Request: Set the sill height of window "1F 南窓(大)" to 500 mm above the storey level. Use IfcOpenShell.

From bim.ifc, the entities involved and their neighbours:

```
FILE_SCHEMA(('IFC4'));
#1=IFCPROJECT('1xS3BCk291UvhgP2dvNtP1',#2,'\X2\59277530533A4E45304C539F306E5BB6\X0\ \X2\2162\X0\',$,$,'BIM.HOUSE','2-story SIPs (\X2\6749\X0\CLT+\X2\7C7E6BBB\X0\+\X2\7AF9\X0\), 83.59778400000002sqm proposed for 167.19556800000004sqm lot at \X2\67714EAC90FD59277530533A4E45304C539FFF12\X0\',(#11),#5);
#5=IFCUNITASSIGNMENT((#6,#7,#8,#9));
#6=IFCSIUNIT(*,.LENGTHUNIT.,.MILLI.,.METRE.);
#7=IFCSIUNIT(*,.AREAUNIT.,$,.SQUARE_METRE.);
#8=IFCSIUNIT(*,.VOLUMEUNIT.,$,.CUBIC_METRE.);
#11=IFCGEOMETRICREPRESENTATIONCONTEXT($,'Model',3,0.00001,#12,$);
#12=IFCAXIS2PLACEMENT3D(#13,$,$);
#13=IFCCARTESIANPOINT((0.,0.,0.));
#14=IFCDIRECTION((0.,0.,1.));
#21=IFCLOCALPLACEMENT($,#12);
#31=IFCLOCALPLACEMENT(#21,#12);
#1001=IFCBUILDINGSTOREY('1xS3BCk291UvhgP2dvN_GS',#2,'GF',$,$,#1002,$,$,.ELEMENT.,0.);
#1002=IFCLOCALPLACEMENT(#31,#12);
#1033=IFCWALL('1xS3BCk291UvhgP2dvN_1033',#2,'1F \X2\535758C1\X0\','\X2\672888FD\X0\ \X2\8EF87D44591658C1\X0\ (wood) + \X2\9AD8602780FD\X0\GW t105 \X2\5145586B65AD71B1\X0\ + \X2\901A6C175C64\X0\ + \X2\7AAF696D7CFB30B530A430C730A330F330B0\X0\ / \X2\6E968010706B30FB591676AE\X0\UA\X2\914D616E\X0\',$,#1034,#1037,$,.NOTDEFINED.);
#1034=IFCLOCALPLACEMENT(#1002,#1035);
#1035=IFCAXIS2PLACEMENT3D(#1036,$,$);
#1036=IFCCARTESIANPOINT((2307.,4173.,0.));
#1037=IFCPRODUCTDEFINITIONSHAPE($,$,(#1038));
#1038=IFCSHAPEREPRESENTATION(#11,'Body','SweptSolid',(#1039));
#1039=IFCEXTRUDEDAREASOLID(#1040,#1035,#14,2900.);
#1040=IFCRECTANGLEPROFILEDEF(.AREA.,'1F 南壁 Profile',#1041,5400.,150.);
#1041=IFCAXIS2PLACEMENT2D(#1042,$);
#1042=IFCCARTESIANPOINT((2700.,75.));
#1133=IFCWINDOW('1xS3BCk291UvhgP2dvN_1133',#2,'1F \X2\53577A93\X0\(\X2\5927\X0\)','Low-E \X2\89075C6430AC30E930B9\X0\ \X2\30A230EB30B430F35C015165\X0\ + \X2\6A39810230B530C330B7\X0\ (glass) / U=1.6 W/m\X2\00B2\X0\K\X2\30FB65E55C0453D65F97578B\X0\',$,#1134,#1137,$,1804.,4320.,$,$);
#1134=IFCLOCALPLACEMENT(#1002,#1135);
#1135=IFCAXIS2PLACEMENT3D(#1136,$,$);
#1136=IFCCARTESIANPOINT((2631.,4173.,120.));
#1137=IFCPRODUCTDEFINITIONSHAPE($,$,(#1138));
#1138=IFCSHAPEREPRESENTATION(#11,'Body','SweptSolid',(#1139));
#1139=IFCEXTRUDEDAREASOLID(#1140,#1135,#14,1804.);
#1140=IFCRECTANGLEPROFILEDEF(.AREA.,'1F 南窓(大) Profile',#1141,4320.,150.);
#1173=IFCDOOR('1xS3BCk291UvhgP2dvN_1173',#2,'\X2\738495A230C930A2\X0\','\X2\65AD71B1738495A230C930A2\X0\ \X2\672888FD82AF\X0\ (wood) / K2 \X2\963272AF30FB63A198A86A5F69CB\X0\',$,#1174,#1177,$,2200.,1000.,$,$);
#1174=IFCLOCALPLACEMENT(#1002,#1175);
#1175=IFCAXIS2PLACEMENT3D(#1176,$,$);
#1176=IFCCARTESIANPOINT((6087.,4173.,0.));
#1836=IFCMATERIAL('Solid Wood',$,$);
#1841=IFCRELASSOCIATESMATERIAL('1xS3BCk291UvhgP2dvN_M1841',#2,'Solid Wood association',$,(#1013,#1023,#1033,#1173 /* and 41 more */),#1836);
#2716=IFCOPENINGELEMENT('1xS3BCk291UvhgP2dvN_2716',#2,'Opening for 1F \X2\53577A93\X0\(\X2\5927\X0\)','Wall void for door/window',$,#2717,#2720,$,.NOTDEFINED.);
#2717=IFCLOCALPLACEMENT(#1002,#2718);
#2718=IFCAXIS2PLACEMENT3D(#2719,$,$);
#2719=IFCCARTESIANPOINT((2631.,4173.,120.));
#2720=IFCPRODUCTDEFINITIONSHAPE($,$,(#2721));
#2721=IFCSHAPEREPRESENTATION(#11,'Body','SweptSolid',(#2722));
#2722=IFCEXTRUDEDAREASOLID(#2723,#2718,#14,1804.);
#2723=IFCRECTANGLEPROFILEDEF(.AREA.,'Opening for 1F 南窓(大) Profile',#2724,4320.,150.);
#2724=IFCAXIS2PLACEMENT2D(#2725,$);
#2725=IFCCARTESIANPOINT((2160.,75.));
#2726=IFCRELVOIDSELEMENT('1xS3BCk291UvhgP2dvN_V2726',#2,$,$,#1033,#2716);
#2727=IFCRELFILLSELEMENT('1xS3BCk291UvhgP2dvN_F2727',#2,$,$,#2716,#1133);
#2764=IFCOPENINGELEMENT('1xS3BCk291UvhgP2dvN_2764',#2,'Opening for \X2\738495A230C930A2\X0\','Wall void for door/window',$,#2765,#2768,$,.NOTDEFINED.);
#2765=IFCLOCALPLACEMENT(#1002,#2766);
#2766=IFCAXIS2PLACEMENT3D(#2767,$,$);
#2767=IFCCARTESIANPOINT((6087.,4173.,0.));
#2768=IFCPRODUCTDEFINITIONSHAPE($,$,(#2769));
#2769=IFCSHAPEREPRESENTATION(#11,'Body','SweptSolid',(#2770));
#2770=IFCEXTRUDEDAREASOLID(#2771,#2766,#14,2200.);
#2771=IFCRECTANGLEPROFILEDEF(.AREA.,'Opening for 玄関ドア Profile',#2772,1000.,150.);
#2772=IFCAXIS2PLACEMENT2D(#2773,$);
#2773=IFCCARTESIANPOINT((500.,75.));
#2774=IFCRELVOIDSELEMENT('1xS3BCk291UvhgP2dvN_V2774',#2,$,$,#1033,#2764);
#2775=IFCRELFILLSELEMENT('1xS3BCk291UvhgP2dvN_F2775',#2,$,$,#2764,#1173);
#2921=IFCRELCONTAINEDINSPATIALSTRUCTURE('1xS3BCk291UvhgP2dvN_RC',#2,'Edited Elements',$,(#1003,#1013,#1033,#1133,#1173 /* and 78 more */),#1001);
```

```python
import numpy as np
import ifcopenshell
import ifcopenshell.api.geometry
import ifcopenshell.geom
import ifcopenshell.util.element
import ifcopenshell.util.placement
import ifcopenshell.util.shape
import ifcopenshell.util.unit

model = ifcopenshell.open("bim.ifc")
unit_scale = ifcopenshell.util.unit.calculate_unit_scale(model)

window = model.by_guid("1xS3BCk291UvhgP2dvN_1133")
opening = window.FillsVoids[0].RelatingOpeningElement
storey = ifcopenshell.util.element.get_container(window, ifc_class="IfcBuildingStorey")
level = ifcopenshell.util.placement.get_local_placement(storey.ObjectPlacement)[2, 3]

# The opening's origin need not be at the sill, so measure its lowest point.
shape = ifcopenshell.geom.create_shape(ifcopenshell.geom.settings(), opening)
bottom = ifcopenshell.util.shape.get_shape_bottom_elevation(shape, shape.geometry) / unit_scale
dz = level + 0.5 / unit_scale - bottom

shift = np.array([0.0, 0.0, dz])
# The window is not placed relative to its opening, so move both.
for product in (opening, window):
    matrix = ifcopenshell.util.placement.get_local_placement(product.ObjectPlacement)
    matrix[:3, 3] += shift
    ifcopenshell.api.geometry.edit_object_placement(model, product=product, matrix=matrix, is_si=False)

print(f"moved by {dz * unit_scale:+.3f} m")

model.write("bim-out.ifc")
```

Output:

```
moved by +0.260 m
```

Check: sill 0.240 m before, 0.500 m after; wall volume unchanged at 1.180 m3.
